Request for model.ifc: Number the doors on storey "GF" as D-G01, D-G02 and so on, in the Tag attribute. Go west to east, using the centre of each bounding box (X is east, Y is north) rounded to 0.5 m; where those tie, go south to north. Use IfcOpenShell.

First a look at what the model holds.

```python
import ifcopenshell
import ifcopenshell.util.element
import ifcopenshell.util.placement

model = ifcopenshell.open("model.ifc")
print(model.schema)
storey = next(s for s in model.by_type("IfcBuildingStorey") if s.Name == "GF")
doors = [e for e in ifcopenshell.util.element.get_decomposition(storey) if e.is_a("IfcDoor")]
for e in sorted(doors, key=lambda e: e.id()):
    origin = ifcopenshell.util.placement.get_local_placement(e.ObjectPlacement)[:3, 3]
    print(e.id(), e.Tag, e.Name, origin.round(2) + 0.0, sep=" | ")
```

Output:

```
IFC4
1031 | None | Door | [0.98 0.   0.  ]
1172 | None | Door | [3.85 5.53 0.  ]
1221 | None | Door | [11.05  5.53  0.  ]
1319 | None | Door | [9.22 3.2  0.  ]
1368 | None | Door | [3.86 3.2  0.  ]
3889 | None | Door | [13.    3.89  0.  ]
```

```python
import ifcopenshell
import ifcopenshell.geom
import ifcopenshell.util.element
import ifcopenshell.util.shape

model = ifcopenshell.open("model.ifc")
settings = ifcopenshell.geom.settings()
settings.set("use-world-coords", True)


def centre(element):
    shape = ifcopenshell.geom.create_shape(settings, element)
    return ifcopenshell.util.shape.get_bbox_centroid(shape.geometry)


storey = next(s for s in model.by_type("IfcBuildingStorey") if s.Name == "GF")
doors = [e for e in ifcopenshell.util.element.get_decomposition(storey) if e.is_a("IfcDoor")]

# Insertion points can sit at a corner or the storey origin, so sort by the geometry (in metres).
centres = {e: centre(e) for e in doors}
doors.sort(key=lambda e: (round(centres[e][0] / 0.5), centres[e][1]))

for i, e in enumerate(doors, start=1):
    number = f"D-G{i:02d}"
    e.Tag = number
    print(e.id(), number)

model.write("model_edited.ifc")
```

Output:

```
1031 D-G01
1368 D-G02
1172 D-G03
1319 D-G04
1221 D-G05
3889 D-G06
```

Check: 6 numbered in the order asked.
